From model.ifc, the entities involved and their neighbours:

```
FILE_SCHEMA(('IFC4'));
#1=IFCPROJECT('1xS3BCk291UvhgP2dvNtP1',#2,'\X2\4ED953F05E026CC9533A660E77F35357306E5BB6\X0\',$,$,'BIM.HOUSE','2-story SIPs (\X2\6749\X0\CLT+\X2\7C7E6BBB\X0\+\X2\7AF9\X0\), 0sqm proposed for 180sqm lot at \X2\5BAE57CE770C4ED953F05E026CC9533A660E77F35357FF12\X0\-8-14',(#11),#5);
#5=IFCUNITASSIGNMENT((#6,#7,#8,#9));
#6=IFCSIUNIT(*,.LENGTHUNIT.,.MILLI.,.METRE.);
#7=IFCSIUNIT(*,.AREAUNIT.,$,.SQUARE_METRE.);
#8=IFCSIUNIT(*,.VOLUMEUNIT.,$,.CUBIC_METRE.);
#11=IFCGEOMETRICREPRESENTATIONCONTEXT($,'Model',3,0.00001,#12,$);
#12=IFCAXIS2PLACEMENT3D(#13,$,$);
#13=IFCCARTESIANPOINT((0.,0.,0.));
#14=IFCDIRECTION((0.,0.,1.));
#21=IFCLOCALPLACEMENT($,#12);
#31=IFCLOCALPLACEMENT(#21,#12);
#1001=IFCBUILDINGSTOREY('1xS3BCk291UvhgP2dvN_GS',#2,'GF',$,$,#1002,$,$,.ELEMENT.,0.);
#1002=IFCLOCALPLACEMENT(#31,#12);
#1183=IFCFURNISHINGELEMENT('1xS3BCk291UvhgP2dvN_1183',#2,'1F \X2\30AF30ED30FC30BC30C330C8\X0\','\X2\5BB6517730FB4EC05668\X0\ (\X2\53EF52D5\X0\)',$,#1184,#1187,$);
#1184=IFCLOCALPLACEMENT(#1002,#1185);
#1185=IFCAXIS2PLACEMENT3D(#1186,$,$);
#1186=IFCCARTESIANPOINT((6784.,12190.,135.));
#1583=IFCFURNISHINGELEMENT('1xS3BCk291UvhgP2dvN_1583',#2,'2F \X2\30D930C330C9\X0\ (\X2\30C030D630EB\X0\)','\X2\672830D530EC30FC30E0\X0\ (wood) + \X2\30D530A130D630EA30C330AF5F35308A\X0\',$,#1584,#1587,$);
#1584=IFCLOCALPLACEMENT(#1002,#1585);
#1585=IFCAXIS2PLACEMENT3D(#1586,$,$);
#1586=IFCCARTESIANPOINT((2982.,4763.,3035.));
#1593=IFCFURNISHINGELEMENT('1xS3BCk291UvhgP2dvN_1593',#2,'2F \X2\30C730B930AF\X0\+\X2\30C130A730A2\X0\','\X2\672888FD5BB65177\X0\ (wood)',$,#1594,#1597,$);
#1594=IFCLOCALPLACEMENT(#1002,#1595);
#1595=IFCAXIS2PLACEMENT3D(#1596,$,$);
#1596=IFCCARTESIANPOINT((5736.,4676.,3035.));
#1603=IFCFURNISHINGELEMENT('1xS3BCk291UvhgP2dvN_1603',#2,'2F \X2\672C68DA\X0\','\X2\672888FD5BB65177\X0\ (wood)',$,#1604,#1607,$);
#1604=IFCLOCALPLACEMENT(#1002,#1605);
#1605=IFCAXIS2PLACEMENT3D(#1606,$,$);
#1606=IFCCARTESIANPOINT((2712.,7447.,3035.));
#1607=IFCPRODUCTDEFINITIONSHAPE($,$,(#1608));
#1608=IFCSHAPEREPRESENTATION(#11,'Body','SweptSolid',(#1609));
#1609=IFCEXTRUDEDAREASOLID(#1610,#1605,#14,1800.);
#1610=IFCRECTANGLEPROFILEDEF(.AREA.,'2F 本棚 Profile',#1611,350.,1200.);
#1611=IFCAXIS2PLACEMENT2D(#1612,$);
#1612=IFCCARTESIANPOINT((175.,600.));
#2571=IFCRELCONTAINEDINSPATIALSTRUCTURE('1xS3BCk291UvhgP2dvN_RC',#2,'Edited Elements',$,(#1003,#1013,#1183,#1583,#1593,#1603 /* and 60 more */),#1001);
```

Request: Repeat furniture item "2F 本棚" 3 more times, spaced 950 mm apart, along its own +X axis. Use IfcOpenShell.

```python
import ifcopenshell
import ifcopenshell.api.geometry
import ifcopenshell.api.root
import ifcopenshell.util.element
import ifcopenshell.util.placement

model = ifcopenshell.open("model.ifc")


def reuse_history(source, copy):
    """copy_class also copies each property set's owner history, people and application; keep the originals."""
    for rel in copy.IsDefinedBy:
        if rel.is_a("IfcRelDefinesByProperties") and (history := rel.RelatingPropertyDefinition.OwnerHistory):
            rel.RelatingPropertyDefinition.OwnerHistory = source.OwnerHistory
            ifcopenshell.util.element.remove_deep2(model, history)


source = model.by_id(1603)
base = ifcopenshell.util.placement.get_local_placement(source.ObjectPlacement)
step = base[:3, 0] * 950.0

for i in range(1, 4):
    copy = ifcopenshell.api.root.copy_class(model, product=source)
    copy.Representation = ifcopenshell.util.element.copy_deep(
        model, source.Representation, exclude=["IfcGeometricRepresentationContext", "IfcRepresentationMap"]
    )
    reuse_history(source, copy)
    matrix = base.copy()
    matrix[:3, 3] += i * step
    print("added at", matrix[:3, 3].round(3) + 0.0)
    ifcopenshell.api.geometry.edit_object_placement(model, product=copy, matrix=matrix, is_si=False)

model.write("model-out.ifc")
```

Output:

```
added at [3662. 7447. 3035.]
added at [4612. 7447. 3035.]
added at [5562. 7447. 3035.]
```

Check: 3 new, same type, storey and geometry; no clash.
